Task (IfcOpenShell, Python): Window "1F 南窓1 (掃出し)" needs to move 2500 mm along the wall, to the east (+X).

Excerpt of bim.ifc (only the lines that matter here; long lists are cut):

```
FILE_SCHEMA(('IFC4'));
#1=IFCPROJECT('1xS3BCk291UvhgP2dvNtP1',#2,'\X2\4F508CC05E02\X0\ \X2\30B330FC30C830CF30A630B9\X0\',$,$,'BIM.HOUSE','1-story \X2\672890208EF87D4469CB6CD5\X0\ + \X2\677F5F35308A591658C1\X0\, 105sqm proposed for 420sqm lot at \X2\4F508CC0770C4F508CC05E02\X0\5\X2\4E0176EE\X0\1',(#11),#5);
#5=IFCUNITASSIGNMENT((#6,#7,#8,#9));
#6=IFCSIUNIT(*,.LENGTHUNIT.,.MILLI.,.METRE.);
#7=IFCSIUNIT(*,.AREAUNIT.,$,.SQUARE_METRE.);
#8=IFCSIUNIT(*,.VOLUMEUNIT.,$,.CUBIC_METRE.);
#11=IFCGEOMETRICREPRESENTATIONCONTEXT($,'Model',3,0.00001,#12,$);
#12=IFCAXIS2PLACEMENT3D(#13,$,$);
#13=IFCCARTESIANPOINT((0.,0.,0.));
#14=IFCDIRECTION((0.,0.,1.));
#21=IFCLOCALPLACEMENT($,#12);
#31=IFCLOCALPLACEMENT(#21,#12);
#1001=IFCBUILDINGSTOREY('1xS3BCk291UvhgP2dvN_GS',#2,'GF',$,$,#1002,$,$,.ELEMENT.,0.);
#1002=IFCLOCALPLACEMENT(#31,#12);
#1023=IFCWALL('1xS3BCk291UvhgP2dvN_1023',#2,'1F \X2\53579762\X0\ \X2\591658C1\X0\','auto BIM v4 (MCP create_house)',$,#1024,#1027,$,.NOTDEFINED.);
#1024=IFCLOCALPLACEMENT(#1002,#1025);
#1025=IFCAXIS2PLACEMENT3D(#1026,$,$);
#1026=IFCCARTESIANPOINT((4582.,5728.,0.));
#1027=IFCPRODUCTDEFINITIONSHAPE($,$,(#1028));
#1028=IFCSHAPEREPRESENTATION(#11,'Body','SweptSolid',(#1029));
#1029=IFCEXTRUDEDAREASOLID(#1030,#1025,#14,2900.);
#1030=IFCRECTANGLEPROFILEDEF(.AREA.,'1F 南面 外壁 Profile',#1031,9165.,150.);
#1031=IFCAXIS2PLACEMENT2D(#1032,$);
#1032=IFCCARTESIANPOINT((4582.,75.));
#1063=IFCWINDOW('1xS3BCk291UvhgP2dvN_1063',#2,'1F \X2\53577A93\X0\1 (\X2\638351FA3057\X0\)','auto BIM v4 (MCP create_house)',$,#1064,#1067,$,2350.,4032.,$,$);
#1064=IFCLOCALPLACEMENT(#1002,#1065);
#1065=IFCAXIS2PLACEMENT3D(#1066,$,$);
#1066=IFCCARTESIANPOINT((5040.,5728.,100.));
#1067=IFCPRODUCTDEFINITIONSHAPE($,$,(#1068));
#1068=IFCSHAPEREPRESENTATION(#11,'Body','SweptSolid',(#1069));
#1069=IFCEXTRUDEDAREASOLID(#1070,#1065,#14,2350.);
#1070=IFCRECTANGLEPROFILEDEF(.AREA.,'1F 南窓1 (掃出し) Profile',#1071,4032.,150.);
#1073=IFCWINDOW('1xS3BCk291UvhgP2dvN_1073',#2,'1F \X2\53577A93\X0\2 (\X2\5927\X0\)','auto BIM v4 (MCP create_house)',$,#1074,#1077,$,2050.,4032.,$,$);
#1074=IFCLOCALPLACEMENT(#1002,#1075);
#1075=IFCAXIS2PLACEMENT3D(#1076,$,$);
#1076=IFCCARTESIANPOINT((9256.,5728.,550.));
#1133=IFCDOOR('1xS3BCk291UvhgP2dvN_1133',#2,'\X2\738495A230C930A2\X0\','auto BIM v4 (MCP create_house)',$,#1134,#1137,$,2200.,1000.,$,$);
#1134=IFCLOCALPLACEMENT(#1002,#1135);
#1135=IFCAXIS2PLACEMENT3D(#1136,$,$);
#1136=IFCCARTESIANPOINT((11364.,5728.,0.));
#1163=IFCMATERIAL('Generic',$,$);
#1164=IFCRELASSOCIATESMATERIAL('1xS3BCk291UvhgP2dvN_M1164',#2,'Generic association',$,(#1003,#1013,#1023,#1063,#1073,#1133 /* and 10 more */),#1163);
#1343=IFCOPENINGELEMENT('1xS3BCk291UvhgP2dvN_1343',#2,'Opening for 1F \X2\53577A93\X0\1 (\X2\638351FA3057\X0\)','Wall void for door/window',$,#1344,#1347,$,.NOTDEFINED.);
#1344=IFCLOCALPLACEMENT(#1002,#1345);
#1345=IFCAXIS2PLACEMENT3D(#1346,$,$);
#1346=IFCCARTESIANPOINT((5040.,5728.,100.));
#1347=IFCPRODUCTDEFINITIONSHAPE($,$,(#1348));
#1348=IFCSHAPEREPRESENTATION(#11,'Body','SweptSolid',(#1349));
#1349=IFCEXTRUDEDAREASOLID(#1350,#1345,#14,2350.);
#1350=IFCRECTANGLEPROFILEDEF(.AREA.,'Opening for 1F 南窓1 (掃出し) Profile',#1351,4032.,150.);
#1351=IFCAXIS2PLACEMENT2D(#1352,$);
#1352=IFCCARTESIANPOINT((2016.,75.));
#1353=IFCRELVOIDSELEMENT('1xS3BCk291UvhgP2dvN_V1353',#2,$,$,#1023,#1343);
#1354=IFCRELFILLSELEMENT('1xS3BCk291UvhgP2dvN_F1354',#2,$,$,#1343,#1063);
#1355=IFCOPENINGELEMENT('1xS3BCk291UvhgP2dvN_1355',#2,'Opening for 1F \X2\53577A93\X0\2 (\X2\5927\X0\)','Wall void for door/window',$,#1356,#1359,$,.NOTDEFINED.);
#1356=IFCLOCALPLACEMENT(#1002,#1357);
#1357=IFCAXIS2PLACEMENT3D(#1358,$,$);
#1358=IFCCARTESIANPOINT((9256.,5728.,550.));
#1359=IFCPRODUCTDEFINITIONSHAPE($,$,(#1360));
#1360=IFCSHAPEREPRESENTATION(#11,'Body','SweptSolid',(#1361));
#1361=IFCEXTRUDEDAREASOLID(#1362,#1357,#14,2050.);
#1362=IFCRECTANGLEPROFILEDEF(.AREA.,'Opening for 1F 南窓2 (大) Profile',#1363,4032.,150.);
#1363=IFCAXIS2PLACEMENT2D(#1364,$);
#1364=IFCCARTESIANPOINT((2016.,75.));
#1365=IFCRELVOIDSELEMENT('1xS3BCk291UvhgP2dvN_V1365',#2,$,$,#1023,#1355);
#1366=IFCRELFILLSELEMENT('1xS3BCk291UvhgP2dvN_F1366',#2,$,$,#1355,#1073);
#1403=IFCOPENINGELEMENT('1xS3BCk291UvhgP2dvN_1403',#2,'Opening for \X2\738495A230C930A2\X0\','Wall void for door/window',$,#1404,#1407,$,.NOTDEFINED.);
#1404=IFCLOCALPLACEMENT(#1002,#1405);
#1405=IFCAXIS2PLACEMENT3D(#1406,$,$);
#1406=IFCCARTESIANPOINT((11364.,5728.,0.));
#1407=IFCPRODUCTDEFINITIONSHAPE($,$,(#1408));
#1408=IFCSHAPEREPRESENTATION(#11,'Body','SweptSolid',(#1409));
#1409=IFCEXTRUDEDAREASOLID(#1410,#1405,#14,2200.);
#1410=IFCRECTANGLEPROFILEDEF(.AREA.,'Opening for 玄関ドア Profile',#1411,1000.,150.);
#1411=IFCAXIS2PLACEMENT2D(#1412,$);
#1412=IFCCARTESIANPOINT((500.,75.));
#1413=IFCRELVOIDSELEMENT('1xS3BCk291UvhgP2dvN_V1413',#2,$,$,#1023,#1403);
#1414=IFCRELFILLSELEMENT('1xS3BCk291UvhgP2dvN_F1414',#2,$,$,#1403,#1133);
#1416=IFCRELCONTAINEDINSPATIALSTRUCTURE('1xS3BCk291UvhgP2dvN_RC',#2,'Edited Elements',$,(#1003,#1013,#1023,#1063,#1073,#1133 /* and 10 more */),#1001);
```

```python
import ifcopenshell
import ifcopenshell.api.geometry
import ifcopenshell.util.placement
import ifcopenshell.util.unit

model = ifcopenshell.open("bim.ifc")
unit_scale = ifcopenshell.util.unit.calculate_unit_scale(model)

window = model.by_guid("1xS3BCk291UvhgP2dvN_1063")
opening = window.FillsVoids[0].RelatingOpeningElement
wall = opening.VoidsElements[0].RelatingBuildingElement

wall_matrix = ifcopenshell.util.placement.get_local_placement(wall.ObjectPlacement)
shift = wall_matrix[:3, 0] * 2.5 / unit_scale
before = ifcopenshell.util.placement.get_local_placement(window.ObjectPlacement)[:3, 3].copy()

# The window is not placed relative to its opening, so move both.
for product in (opening, window):
    matrix = ifcopenshell.util.placement.get_local_placement(product.ObjectPlacement)
    matrix[:3, 3] += shift
    ifcopenshell.api.geometry.edit_object_placement(model, product=product, matrix=matrix, is_si=False)

after = ifcopenshell.util.placement.get_local_placement(window.ObjectPlacement)[:3, 3]
print("window moved by", (after - before).round(3) + 0.0)

model.write("bim_updated.ifc")
```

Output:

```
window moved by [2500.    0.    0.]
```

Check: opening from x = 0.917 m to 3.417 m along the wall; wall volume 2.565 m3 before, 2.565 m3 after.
